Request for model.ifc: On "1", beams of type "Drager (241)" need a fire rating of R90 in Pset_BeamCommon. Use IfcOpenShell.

First a look at what the model holds.

```python
import ifcopenshell
import ifcopenshell.util.element

model = ifcopenshell.open("model.ifc")
print(model.schema)
storey = next(s for s in model.by_type("IfcBuildingStorey") if s.Name == "1")
beams = [e for e in ifcopenshell.util.element.get_decomposition(storey) if e.is_a("IfcBeam")]
seen = {}
for e in beams:
    element_type = ifcopenshell.util.element.get_type(e)
    key = (element_type.Name if element_type != e and element_type else None, ifcopenshell.util.element.get_pset(e, "Pset_BeamCommon", "FireRating"))
    seen[key] = seen.get(key, 0) + 1
for (name, value), count in sorted(seen.items(), key=str):
    print(count, "x", name, "|", value)
```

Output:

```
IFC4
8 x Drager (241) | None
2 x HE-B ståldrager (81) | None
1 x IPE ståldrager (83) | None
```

```python
import ifcopenshell
import ifcopenshell.api.pset
import ifcopenshell.util.element

model = ifcopenshell.open("model.ifc")

storey = next(s for s in model.by_type("IfcBuildingStorey") if s.Name == "1")
beams = [e for e in ifcopenshell.util.element.get_decomposition(storey) if e.is_a("IfcBeam")]

count = 0
for e in beams:
    element_type = ifcopenshell.util.element.get_type(e)
    if element_type in (None, e) or element_type.Name != "Drager (241)":
        continue
    # add_pset returns the element's existing set when there is one.
    pset = ifcopenshell.api.pset.add_pset(model, product=e, name="Pset_BeamCommon")
    ifcopenshell.api.pset.edit_pset(model, pset=pset, properties={"FireRating": "R90"})
    count += 1

print(count, "beams updated")

model.write("model_edited.ifc")
```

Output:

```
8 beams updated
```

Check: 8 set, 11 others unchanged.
